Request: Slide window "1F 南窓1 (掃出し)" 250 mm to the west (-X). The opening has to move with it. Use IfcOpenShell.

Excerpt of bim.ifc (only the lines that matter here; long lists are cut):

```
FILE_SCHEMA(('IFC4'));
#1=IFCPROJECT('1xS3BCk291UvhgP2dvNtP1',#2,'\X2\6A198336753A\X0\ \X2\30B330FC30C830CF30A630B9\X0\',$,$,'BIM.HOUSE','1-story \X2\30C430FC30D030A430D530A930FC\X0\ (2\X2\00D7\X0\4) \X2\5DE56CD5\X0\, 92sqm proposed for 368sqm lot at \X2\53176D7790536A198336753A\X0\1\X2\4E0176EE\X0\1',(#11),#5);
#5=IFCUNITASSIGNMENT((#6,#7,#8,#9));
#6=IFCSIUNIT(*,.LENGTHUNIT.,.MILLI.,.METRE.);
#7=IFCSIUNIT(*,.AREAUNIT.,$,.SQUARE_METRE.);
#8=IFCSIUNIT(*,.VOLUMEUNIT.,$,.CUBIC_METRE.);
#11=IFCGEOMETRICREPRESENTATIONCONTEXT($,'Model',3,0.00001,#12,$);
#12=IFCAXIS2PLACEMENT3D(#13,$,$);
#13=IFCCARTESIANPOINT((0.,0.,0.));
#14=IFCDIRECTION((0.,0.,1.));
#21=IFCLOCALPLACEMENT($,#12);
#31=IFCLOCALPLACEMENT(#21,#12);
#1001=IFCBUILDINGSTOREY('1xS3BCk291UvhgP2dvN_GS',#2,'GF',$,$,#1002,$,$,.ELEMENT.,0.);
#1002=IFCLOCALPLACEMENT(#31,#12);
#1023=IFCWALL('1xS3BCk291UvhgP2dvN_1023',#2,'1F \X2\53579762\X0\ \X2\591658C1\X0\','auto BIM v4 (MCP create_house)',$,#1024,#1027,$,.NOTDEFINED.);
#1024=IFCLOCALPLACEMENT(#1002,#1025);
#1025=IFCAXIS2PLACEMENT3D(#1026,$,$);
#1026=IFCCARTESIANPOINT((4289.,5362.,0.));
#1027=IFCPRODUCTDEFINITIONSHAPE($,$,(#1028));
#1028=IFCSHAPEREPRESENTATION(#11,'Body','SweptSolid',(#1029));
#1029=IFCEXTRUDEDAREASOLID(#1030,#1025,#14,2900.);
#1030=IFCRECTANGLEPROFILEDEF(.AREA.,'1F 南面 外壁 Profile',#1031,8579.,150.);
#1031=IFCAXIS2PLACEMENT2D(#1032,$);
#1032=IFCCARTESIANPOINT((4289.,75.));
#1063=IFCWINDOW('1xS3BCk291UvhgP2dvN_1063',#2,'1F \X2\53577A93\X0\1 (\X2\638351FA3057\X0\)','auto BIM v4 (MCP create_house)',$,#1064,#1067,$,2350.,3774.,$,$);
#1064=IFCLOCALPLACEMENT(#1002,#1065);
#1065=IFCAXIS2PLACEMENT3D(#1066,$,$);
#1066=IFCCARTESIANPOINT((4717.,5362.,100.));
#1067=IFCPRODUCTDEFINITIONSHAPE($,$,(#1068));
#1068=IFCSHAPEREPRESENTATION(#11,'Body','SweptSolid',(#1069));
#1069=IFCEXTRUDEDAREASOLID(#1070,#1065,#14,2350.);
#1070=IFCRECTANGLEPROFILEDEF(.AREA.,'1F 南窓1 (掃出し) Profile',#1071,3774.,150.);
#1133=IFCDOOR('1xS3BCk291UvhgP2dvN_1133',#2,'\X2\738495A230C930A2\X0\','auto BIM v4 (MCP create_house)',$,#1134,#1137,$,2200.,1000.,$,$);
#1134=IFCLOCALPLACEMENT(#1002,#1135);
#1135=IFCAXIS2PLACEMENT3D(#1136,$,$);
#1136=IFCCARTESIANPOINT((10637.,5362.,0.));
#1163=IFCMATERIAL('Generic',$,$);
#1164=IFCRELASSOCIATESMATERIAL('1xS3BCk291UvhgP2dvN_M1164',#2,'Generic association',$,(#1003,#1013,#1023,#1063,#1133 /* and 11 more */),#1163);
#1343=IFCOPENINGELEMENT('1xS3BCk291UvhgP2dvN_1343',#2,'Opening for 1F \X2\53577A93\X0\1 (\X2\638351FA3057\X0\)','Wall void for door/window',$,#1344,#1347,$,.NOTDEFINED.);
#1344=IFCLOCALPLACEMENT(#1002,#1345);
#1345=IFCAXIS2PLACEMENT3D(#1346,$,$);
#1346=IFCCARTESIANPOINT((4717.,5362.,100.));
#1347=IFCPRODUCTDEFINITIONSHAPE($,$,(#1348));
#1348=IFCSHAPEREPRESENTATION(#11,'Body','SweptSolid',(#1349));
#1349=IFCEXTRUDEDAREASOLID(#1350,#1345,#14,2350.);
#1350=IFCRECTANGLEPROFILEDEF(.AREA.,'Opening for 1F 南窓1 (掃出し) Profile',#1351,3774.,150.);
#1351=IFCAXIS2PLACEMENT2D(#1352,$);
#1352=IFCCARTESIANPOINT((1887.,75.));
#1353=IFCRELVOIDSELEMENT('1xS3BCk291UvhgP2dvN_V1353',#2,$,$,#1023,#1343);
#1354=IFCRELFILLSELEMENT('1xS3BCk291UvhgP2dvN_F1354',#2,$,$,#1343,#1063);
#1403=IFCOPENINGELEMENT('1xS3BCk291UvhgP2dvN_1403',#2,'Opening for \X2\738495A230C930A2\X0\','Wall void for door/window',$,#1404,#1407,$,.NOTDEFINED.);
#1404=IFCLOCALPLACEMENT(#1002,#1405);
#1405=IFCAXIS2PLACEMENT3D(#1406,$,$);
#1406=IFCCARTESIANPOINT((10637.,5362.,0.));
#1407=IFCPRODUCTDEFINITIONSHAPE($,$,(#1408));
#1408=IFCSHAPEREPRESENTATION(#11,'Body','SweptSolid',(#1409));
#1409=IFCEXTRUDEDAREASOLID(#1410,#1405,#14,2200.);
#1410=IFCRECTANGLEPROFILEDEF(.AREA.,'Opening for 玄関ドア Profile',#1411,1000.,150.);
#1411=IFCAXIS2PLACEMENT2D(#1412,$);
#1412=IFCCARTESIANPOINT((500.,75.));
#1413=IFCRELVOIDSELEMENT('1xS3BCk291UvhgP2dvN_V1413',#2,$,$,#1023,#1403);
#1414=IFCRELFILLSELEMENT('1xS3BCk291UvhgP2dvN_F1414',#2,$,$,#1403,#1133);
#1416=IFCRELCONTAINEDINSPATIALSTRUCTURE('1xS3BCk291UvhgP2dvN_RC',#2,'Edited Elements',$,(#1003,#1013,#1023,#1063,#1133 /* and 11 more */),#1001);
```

```python
import ifcopenshell
import ifcopenshell.api.geometry
import ifcopenshell.util.placement
import ifcopenshell.util.unit

model = ifcopenshell.open("bim.ifc")
unit_scale = ifcopenshell.util.unit.calculate_unit_scale(model)

window = model.by_guid("1xS3BCk291UvhgP2dvN_1063")
opening = window.FillsVoids[0].RelatingOpeningElement
wall = opening.VoidsElements[0].RelatingBuildingElement

wall_matrix = ifcopenshell.util.placement.get_local_placement(wall.ObjectPlacement)
shift = wall_matrix[:3, 0] * -0.25 / unit_scale
before = ifcopenshell.util.placement.get_local_placement(window.ObjectPlacement)[:3, 3].copy()

# The window is not placed relative to its opening, so move both.
for product in (opening, window):
    matrix = ifcopenshell.util.placement.get_local_placement(product.ObjectPlacement)
    matrix[:3, 3] += shift
    ifcopenshell.api.geometry.edit_object_placement(model, product=product, matrix=matrix, is_si=False)

after = ifcopenshell.util.placement.get_local_placement(window.ObjectPlacement)[:3, 3]
print("window moved by", (after - before).round(3) + 0.0)

model.write("bim_updated.ifc")
```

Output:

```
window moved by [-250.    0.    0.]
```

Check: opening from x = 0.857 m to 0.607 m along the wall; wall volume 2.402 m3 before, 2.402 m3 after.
